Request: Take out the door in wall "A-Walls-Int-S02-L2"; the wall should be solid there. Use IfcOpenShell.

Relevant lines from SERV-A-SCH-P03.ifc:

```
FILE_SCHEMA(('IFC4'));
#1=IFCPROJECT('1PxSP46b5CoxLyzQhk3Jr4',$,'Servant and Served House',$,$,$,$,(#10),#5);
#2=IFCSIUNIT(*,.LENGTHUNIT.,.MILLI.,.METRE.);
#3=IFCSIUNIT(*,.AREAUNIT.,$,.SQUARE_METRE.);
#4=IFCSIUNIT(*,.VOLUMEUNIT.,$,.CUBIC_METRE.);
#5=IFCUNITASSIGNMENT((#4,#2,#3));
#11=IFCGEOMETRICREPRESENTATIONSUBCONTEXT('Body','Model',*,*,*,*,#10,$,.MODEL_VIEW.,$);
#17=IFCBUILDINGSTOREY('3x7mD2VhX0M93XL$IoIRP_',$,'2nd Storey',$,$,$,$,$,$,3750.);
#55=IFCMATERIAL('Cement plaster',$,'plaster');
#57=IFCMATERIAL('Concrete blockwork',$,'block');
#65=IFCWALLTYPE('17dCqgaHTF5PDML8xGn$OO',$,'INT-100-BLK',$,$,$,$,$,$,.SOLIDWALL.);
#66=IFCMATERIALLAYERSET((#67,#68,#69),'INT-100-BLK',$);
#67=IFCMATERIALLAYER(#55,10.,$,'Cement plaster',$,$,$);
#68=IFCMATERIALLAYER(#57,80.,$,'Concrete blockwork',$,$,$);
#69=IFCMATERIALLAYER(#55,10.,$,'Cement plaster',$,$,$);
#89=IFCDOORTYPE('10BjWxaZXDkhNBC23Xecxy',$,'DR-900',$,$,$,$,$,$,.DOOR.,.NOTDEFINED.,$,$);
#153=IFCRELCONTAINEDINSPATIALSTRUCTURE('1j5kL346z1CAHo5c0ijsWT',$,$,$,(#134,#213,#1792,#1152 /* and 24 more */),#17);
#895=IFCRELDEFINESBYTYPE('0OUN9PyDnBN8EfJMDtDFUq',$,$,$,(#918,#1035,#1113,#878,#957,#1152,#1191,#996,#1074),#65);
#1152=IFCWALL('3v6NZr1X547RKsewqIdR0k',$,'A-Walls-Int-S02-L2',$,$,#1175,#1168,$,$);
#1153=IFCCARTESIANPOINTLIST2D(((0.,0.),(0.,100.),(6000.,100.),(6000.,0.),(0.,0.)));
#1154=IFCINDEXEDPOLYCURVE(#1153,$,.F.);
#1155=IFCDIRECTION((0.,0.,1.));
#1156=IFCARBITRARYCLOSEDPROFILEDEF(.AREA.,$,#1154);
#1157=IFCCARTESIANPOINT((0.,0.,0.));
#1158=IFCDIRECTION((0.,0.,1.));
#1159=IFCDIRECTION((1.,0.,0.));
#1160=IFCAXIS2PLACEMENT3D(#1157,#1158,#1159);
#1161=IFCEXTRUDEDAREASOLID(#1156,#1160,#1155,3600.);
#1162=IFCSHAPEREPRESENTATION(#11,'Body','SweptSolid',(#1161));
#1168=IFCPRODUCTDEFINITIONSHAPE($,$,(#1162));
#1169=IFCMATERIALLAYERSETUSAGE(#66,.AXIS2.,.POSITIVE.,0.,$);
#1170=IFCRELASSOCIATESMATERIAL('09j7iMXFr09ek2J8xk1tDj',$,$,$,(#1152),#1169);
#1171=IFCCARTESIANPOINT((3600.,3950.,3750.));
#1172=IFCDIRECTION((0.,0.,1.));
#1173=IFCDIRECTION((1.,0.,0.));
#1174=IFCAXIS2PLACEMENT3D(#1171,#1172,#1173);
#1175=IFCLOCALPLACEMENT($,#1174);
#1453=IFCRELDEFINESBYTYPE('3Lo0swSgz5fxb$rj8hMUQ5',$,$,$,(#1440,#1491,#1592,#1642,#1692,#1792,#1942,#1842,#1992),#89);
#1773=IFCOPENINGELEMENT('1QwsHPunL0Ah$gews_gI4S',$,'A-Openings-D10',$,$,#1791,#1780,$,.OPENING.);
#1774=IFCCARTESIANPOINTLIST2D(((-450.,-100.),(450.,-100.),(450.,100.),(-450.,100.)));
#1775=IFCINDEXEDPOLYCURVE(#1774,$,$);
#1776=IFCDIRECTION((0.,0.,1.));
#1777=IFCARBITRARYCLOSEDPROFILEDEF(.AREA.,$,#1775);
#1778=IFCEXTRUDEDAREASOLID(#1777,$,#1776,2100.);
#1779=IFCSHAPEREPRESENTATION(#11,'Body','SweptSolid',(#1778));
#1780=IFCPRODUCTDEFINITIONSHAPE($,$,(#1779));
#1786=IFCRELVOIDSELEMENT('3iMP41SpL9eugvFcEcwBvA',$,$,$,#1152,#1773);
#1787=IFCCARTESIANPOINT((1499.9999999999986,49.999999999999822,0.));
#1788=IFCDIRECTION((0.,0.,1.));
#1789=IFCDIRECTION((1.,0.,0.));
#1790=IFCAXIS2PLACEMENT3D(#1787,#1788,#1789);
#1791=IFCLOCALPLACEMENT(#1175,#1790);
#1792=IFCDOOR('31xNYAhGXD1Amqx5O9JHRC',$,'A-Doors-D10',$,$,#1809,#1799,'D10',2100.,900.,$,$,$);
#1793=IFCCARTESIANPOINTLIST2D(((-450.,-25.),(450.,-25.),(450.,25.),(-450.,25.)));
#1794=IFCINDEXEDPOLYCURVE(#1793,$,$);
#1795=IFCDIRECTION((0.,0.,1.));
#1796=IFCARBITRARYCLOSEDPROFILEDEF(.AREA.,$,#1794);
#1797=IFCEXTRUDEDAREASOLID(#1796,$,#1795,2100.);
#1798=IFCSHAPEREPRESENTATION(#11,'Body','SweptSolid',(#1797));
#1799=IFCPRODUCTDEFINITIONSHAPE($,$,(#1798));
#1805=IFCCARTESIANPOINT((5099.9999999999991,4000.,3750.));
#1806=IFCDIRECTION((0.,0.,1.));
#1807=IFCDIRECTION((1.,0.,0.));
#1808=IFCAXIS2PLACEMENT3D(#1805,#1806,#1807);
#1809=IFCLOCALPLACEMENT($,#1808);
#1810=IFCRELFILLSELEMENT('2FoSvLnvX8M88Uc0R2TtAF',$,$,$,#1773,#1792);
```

```python
import ifcopenshell
import ifcopenshell.api.feature
import ifcopenshell.api.root
import ifcopenshell.geom
import ifcopenshell.util.shape

model = ifcopenshell.open("SERV-A-SCH-P03.ifc")
settings = ifcopenshell.geom.settings()


def volume(element):
    """Net volume in cubic metres, openings subtracted."""
    shape = ifcopenshell.geom.create_shape(settings, element)
    return ifcopenshell.util.shape.get_volume(shape.geometry)


door = model.by_guid("31xNYAhGXD1Amqx5O9JHRC")
opening = door.FillsVoids[0].RelatingOpeningElement
wall = opening.VoidsElements[0].RelatingBuildingElement
before = volume(wall)

ifcopenshell.api.root.remove_product(model, product=door)
ifcopenshell.api.feature.remove_feature(model, feature=opening)

after = volume(wall)

print(f"wall volume {before:.3f} -> {after:.3f} m3")

model.write("SERV-A-SCH-P03_rev.ifc")
```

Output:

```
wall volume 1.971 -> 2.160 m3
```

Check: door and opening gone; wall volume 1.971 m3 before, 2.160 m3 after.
